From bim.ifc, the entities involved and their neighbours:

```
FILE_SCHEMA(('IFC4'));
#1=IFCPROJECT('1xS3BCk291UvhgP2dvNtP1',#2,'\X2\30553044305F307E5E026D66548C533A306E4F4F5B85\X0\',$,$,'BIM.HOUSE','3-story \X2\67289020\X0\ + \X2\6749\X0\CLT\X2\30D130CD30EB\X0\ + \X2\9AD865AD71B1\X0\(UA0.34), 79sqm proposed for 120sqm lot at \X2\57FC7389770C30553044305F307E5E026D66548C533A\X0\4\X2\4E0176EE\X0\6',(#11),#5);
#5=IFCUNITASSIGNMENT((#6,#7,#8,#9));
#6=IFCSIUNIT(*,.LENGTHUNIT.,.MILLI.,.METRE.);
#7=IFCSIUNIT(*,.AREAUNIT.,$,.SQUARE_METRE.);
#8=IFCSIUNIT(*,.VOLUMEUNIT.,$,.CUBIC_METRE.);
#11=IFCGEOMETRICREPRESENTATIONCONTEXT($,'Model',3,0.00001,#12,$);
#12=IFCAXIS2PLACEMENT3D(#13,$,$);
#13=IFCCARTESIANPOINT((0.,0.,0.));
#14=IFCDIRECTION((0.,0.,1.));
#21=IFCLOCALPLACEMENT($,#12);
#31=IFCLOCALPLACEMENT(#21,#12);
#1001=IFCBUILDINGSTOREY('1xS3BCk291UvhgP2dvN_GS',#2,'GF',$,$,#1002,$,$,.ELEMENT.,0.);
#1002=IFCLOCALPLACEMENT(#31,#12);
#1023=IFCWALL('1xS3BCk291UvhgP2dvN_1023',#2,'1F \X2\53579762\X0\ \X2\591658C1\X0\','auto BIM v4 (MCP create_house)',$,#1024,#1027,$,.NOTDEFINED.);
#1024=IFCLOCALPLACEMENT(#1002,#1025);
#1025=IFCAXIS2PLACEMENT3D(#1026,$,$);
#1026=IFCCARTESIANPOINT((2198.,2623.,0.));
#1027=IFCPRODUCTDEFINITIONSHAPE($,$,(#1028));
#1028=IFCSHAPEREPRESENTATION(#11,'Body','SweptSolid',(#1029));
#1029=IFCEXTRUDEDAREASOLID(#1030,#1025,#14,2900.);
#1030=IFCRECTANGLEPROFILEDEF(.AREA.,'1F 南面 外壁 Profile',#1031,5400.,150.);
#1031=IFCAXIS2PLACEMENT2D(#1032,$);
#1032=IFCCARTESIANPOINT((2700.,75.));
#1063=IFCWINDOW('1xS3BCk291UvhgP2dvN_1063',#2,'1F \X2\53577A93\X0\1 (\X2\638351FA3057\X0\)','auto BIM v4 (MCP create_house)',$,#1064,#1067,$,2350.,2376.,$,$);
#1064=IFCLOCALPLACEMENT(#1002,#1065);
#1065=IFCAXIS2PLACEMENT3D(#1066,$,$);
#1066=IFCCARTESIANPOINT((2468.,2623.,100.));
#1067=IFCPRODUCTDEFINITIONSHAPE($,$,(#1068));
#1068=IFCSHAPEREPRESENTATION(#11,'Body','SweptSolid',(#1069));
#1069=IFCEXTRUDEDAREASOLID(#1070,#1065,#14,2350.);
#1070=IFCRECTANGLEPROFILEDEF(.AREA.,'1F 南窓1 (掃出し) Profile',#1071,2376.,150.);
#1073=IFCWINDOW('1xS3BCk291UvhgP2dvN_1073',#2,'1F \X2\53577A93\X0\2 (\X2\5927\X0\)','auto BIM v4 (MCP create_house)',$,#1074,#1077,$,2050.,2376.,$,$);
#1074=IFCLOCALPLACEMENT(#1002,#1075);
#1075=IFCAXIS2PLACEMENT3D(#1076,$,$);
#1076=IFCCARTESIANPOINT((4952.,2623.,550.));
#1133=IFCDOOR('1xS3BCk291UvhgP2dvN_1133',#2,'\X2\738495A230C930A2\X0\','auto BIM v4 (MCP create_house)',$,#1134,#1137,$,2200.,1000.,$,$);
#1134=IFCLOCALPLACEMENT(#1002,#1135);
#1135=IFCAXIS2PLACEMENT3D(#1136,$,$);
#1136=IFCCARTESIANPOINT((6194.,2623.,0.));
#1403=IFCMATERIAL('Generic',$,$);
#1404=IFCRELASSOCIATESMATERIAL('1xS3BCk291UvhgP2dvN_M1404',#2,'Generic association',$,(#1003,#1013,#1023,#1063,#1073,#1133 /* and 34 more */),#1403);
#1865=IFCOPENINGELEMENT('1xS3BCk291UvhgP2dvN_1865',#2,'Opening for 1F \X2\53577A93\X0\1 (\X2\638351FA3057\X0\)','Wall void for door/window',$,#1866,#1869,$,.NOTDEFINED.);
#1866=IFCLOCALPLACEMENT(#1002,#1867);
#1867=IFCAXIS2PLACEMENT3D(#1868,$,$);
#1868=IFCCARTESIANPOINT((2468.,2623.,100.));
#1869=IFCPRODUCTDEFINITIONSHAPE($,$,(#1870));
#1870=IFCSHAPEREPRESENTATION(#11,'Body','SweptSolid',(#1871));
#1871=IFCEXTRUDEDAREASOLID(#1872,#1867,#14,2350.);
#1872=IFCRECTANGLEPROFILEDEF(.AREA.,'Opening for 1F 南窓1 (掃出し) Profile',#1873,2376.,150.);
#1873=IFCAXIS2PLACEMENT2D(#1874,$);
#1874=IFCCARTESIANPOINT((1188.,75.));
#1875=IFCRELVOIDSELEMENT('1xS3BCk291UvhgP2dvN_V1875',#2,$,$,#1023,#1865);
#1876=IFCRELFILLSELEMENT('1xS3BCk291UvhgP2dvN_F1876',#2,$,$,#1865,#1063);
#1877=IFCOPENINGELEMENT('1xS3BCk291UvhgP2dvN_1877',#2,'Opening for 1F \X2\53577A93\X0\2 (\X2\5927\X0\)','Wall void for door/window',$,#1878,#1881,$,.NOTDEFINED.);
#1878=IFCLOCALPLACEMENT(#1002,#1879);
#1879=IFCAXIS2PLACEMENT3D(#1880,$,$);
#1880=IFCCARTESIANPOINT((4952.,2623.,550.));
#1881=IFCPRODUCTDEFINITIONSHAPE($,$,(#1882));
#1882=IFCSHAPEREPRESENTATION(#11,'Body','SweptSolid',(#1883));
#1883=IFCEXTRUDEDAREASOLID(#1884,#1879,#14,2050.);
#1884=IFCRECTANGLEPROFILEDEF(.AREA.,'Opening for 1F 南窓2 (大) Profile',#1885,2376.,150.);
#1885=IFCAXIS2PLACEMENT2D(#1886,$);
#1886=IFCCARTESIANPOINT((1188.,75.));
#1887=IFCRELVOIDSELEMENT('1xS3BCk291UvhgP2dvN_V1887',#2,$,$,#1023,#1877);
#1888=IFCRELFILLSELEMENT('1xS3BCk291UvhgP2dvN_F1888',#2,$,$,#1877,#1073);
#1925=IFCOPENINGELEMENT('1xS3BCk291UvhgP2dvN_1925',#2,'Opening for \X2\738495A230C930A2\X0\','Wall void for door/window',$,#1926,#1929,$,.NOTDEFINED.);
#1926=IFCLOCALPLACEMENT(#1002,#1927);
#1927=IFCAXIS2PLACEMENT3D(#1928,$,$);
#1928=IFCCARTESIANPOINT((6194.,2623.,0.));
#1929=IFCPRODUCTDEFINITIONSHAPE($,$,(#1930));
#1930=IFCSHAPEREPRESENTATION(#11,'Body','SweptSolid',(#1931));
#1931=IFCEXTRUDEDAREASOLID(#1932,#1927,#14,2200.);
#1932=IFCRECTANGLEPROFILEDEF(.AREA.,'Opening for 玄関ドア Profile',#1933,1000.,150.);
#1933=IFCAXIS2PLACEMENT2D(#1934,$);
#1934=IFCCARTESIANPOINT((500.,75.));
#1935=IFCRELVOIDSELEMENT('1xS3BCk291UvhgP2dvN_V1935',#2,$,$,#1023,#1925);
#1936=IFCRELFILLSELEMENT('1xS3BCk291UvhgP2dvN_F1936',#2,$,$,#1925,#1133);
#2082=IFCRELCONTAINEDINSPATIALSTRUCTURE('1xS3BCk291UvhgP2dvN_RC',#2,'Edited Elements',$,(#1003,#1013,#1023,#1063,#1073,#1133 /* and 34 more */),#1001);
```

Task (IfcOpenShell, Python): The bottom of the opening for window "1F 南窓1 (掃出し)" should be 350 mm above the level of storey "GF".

```python
import numpy as np
import ifcopenshell
import ifcopenshell.api.geometry
import ifcopenshell.geom
import ifcopenshell.util.element
import ifcopenshell.util.placement
import ifcopenshell.util.shape
import ifcopenshell.util.unit

model = ifcopenshell.open("bim.ifc")
unit_scale = ifcopenshell.util.unit.calculate_unit_scale(model)

window = model.by_guid("1xS3BCk291UvhgP2dvN_1063")
opening = window.FillsVoids[0].RelatingOpeningElement
storey = ifcopenshell.util.element.get_container(window, ifc_class="IfcBuildingStorey")
level = ifcopenshell.util.placement.get_local_placement(storey.ObjectPlacement)[2, 3]

# The opening's origin need not be at the sill, so measure its lowest point.
shape = ifcopenshell.geom.create_shape(ifcopenshell.geom.settings(), opening)
bottom = ifcopenshell.util.shape.get_shape_bottom_elevation(shape, shape.geometry) / unit_scale
dz = level + 350.0 - bottom

shift = np.array([0.0, 0.0, dz])
# The window is not placed relative to its opening, so move both.
for product in (opening, window):
    matrix = ifcopenshell.util.placement.get_local_placement(product.ObjectPlacement)
    matrix[:3, 3] += shift
    ifcopenshell.api.geometry.edit_object_placement(model, product=product, matrix=matrix, is_si=False)

print(f"moved by {dz * unit_scale:+.3f} m")

model.write("bim_updated.ifc")
```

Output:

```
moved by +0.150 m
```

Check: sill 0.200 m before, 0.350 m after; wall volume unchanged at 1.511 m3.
